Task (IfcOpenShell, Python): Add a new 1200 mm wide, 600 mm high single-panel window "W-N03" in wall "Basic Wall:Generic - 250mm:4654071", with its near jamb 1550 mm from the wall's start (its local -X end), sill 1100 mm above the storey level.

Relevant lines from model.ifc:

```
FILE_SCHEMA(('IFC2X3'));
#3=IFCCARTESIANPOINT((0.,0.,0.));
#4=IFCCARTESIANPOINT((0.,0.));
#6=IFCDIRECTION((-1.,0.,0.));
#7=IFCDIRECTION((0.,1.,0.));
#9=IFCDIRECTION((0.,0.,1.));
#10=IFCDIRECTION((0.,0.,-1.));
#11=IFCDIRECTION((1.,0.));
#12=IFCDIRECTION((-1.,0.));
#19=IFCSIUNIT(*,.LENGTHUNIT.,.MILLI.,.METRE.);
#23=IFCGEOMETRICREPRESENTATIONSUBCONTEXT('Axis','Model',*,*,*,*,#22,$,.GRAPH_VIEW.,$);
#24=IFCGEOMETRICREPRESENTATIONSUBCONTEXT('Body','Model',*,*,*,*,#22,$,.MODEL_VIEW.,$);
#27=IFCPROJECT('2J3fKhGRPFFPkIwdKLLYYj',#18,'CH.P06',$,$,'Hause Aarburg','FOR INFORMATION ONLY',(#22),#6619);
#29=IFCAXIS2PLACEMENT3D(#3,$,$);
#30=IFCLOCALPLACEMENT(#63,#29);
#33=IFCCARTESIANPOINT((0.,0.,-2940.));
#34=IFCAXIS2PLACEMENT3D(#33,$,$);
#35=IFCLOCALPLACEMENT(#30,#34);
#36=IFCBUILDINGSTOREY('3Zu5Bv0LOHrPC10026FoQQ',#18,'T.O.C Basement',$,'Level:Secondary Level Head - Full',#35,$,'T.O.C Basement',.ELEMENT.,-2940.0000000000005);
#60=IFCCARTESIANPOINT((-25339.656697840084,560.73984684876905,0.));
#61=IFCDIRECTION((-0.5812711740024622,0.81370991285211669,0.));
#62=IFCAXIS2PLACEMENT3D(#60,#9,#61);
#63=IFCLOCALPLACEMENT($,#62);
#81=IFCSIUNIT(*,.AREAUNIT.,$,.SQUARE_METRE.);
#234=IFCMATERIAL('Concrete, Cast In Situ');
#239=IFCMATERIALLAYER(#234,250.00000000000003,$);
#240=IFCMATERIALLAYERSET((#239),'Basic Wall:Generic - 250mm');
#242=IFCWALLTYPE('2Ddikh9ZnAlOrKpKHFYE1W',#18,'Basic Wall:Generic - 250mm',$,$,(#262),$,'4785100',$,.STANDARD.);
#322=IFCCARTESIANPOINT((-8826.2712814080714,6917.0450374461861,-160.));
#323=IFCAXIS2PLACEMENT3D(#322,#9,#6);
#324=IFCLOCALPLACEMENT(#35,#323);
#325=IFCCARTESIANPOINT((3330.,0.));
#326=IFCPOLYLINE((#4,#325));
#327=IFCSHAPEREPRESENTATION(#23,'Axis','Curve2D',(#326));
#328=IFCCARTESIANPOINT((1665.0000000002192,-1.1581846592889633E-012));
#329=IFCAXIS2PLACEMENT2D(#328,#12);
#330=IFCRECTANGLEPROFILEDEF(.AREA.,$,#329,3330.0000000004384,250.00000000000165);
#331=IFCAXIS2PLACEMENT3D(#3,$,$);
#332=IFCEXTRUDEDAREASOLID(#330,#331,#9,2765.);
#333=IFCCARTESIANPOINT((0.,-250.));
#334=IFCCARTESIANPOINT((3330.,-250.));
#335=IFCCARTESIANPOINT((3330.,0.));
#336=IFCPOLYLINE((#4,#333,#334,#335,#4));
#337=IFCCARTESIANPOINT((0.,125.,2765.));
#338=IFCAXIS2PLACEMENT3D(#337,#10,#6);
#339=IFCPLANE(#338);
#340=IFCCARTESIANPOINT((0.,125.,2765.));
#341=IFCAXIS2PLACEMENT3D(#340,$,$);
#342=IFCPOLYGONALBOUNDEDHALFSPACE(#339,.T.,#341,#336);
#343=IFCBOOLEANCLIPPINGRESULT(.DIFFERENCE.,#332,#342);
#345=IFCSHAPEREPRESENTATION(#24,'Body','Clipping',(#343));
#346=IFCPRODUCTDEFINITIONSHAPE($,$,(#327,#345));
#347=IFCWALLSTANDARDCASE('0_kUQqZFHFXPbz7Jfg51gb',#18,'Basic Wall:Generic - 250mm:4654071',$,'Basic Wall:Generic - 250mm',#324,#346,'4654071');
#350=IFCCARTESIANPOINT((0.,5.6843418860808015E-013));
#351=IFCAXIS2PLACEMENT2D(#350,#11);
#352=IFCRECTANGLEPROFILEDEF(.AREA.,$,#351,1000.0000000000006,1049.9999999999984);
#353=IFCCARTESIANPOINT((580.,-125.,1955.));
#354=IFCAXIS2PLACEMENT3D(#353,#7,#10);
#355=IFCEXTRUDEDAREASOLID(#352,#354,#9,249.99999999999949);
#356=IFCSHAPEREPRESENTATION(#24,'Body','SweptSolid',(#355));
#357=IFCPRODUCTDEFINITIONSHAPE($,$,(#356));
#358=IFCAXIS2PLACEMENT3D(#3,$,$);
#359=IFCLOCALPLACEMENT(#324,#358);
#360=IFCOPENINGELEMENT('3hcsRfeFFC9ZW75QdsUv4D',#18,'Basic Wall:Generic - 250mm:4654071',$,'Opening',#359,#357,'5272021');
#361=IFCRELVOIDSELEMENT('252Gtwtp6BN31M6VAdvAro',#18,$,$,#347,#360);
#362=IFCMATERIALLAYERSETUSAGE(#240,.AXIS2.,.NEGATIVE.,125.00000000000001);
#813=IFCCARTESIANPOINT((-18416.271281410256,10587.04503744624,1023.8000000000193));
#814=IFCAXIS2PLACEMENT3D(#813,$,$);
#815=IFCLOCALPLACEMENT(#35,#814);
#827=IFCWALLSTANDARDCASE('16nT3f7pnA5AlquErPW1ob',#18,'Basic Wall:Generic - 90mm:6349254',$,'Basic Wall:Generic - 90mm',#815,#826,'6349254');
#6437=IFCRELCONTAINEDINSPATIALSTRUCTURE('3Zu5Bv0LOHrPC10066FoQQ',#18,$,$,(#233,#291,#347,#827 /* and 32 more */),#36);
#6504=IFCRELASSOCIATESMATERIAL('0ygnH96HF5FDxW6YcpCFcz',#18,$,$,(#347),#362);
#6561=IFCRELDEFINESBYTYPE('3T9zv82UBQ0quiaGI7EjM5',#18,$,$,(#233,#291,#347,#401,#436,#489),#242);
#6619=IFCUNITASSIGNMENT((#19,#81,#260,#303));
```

```python
import numpy as np
import ifcopenshell
import ifcopenshell.api.feature
import ifcopenshell.api.geometry
import ifcopenshell.api.root
import ifcopenshell.api.spatial
import ifcopenshell.api.type
import ifcopenshell.geom
import ifcopenshell.util.element
import ifcopenshell.util.placement
import ifcopenshell.util.representation
import ifcopenshell.util.shape
import ifcopenshell.util.unit

model = ifcopenshell.open("model.ifc")
unit_scale = ifcopenshell.util.unit.calculate_unit_scale(model)
settings = ifcopenshell.geom.settings()


def volume(element):
    """Net volume in cubic metres, openings subtracted."""
    shape = ifcopenshell.geom.create_shape(settings, element)
    return ifcopenshell.util.shape.get_volume(shape.geometry)


wall = model.by_id(347)
storey = ifcopenshell.util.element.get_container(wall, ifc_class="IfcBuildingStorey")
context = ifcopenshell.util.representation.get_context(model, "Model", "Body", "MODEL_VIEW")
before = volume(wall)

width, height, from_end, sill = 1.2, 0.6, 1.55, 1.1  # metres

# The wall runs along its own X axis, and the end named is its -X end.
wall_shape = ifcopenshell.geom.create_shape(settings, wall)
x, y, z = ifcopenshell.util.shape.get_vertices(wall_shape.geometry).T
start = x.min() + from_end
face, thickness = float(y.min()), float(y.max() - y.min())
wall_matrix = ifcopenshell.util.placement.get_local_placement(wall.ObjectPlacement)
level = ifcopenshell.util.placement.get_local_placement(storey.ObjectPlacement)[2, 3]


def in_wall(x, y):
    """Placement at x, y metres in the wall's axes, at sill height."""
    matrix = wall_matrix.copy()
    matrix[:, 3] = wall_matrix @ np.array([x / unit_scale, y / unit_scale, 0.0, 1.0])
    matrix[2, 3] = level + sill / unit_scale
    return matrix


# Opening: a box that overshoots both wall faces by 50 mm.
opening = ifcopenshell.api.root.create_entity(model, ifc_class="IfcOpeningElement")
box = ifcopenshell.api.geometry.add_wall_representation(
    model, context=context, length=width, height=height, thickness=thickness + 0.1
)
ifcopenshell.api.geometry.assign_representation(model, product=opening, representation=box)
ifcopenshell.api.geometry.edit_object_placement(model, product=opening, matrix=in_wall(start, face - 0.05), is_si=False)
ifcopenshell.api.feature.add_feature(model, feature=opening, element=wall)

window = ifcopenshell.api.root.create_entity(model, ifc_class="IfcWindow", name="W-N03")
window.OverallWidth, window.OverallHeight = width / unit_scale, height / unit_scale
body = ifcopenshell.api.geometry.add_window_representation(
    model,
    context=context,
    overall_width=window.OverallWidth,
    overall_height=window.OverallHeight,
    partition_type="SINGLE_PANEL",
)
ifcopenshell.api.geometry.assign_representation(model, product=window, representation=body)
ifcopenshell.api.spatial.assign_container(model, products=[window], relating_structure=storey)
fills = ifcopenshell.api.feature.add_filling(model, opening=opening, element=window)
fills.OwnerHistory = window.OwnerHistory  # required in IFC2X3

# IFC2X3 keeps the operation on the window style.
style = ifcopenshell.api.root.create_entity(model, ifc_class="IfcWindowStyle", name="W-N03")
style.OperationType, style.ConstructionType = "SINGLE_PANEL", "NOTDEFINED"
style.ParameterTakesPrecedence = style.Sizeable = False
ifcopenshell.api.type.assign_type(model, related_objects=[window], relating_type=style)

# Centre the window in the wall's thickness.
ifcopenshell.api.geometry.edit_object_placement(model, product=window, matrix=in_wall(start, face), is_si=False)
window_shape = ifcopenshell.geom.create_shape(settings, window)
depth = ifcopenshell.util.shape.get_vertices(window_shape.geometry)[:, 1]
offset = face + thickness / 2 - (depth.min() + depth.max()) / 2
ifcopenshell.api.geometry.edit_object_placement(model, product=window, matrix=in_wall(start, offset), is_si=False)

after = volume(wall)

print(f"wall volume {before:.3f} -> {after:.3f} m3")

model.write("model_rev.ifc")
```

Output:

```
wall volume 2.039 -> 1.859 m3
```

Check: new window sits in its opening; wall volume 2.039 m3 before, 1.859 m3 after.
